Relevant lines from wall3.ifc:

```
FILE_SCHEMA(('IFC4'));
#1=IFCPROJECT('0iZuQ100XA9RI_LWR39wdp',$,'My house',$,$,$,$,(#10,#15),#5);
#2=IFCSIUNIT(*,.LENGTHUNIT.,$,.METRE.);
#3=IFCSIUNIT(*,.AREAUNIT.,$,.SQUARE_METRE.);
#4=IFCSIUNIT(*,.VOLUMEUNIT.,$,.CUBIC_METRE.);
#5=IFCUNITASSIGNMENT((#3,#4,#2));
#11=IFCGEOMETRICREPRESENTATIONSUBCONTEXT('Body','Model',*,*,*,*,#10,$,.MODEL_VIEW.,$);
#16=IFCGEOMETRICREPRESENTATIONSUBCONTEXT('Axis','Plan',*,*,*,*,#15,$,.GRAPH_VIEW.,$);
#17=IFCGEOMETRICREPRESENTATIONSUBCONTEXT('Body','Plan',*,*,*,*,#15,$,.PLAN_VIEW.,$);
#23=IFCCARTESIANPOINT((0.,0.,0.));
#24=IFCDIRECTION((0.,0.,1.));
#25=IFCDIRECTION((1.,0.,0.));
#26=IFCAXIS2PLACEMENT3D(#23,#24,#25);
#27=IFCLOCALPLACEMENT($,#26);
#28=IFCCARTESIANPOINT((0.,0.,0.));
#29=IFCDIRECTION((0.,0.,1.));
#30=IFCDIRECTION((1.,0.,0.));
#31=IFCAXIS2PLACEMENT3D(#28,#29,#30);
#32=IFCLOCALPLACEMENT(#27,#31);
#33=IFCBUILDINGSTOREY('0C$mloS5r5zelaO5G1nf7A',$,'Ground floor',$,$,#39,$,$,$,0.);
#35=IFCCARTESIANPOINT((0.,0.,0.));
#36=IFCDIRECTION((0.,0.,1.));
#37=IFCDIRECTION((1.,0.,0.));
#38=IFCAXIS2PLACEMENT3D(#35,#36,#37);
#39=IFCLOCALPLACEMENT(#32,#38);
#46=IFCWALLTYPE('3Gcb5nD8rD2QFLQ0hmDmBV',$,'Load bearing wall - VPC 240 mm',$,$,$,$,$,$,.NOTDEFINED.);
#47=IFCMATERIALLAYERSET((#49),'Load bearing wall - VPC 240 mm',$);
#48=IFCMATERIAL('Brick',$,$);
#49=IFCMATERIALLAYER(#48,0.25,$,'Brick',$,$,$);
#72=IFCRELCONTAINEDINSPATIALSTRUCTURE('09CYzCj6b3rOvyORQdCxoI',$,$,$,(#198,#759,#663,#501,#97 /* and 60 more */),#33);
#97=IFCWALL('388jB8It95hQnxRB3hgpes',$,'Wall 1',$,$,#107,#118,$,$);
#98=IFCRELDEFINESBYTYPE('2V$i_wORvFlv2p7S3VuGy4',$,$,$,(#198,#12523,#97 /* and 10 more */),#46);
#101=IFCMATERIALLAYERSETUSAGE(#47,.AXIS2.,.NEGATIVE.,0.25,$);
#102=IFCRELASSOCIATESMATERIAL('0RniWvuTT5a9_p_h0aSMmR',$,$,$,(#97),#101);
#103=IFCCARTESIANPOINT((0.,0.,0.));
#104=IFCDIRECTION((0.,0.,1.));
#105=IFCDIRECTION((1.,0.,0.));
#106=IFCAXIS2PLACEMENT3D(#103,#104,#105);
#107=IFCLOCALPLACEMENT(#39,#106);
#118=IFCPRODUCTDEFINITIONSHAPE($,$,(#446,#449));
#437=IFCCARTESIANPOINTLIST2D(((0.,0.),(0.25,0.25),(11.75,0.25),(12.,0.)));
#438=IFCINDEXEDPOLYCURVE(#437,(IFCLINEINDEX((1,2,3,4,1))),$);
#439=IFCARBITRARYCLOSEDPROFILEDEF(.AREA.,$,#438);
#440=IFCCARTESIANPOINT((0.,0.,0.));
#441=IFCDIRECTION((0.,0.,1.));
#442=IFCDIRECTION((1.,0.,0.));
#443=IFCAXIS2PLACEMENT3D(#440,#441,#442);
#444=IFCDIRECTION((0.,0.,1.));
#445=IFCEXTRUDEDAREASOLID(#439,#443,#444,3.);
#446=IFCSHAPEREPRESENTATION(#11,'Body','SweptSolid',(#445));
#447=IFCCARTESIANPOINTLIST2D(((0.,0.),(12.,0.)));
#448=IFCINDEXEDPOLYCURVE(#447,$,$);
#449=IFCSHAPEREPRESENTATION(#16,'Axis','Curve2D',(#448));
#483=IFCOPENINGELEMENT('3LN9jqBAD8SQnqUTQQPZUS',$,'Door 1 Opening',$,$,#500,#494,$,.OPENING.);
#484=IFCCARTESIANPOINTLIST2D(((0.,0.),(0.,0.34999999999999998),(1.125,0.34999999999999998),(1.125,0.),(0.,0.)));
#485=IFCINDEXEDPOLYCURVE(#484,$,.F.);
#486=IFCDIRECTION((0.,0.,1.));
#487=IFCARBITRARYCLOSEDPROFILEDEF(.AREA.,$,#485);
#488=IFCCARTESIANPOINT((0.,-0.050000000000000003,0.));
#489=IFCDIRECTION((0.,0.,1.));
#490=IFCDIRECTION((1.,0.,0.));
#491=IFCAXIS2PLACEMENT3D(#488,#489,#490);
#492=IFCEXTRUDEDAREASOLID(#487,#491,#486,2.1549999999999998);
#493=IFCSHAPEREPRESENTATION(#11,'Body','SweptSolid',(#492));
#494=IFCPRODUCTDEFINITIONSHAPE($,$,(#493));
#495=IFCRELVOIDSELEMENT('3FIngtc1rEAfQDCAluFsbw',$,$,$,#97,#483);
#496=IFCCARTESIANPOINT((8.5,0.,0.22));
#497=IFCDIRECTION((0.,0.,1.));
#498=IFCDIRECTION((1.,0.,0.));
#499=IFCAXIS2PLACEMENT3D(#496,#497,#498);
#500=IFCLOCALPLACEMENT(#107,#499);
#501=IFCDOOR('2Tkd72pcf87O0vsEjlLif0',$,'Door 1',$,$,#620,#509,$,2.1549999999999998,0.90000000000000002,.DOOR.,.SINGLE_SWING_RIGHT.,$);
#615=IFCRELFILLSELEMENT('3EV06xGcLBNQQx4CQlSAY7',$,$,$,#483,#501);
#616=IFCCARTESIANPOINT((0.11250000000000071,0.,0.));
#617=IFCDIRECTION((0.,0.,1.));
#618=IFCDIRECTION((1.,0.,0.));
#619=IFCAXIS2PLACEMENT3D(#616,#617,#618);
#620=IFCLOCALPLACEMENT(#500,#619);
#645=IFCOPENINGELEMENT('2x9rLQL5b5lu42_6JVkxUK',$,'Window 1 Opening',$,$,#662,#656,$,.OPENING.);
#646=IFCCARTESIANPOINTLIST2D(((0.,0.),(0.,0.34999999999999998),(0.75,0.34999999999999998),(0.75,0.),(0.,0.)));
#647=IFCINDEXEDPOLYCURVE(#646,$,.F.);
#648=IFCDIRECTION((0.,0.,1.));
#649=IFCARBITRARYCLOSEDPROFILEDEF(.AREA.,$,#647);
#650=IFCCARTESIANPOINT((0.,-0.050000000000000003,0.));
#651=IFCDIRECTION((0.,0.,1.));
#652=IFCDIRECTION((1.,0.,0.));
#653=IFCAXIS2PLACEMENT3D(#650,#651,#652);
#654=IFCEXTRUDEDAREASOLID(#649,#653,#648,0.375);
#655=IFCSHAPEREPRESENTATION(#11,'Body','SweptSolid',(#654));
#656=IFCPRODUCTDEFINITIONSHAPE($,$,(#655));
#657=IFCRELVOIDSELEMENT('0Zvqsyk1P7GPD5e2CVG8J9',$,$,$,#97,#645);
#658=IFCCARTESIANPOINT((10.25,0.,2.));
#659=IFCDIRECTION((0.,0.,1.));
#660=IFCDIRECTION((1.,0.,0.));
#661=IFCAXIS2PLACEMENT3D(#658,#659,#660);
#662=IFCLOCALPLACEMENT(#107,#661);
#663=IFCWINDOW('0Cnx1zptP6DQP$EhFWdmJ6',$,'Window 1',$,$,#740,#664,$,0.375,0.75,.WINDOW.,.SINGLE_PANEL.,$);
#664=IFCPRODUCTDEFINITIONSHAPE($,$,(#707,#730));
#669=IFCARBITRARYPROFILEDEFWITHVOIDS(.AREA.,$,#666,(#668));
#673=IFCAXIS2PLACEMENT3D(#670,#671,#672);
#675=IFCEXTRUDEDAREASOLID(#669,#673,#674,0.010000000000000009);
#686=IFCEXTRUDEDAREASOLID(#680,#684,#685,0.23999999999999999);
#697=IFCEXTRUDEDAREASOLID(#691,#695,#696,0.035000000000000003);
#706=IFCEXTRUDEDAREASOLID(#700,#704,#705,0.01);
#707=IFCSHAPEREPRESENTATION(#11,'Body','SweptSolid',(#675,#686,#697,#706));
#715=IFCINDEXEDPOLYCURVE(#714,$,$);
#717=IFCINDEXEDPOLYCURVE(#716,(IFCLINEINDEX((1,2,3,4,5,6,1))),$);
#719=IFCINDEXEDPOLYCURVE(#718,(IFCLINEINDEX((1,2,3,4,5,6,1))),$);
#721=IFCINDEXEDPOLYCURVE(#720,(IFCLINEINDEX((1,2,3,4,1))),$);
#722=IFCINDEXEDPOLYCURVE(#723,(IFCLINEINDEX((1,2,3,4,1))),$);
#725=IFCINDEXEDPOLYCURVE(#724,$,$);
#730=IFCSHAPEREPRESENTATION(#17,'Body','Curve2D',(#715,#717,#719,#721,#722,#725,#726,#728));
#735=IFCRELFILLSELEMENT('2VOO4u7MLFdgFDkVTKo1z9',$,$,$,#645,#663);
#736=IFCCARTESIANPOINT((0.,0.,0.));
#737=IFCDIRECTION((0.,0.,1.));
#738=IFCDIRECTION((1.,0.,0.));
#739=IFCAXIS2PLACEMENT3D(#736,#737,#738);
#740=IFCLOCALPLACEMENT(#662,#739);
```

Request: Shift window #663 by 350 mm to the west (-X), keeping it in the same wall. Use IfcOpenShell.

```python
import ifcopenshell
import ifcopenshell.api.geometry
import ifcopenshell.util.placement
import ifcopenshell.util.unit

model = ifcopenshell.open("wall3.ifc")
unit_scale = ifcopenshell.util.unit.calculate_unit_scale(model)

window = model.by_id(663)
opening = window.FillsVoids[0].RelatingOpeningElement
wall = opening.VoidsElements[0].RelatingBuildingElement

wall_matrix = ifcopenshell.util.placement.get_local_placement(wall.ObjectPlacement)
shift = wall_matrix[:3, 0] * -0.35 / unit_scale
before = ifcopenshell.util.placement.get_local_placement(window.ObjectPlacement)[:3, 3].copy()

# The window is placed relative to its opening, so it follows when the opening moves.
matrix = ifcopenshell.util.placement.get_local_placement(opening.ObjectPlacement)
matrix[:3, 3] += shift
ifcopenshell.api.geometry.edit_object_placement(
    model, product=opening, matrix=matrix, is_si=False, should_transform_children=True
)

after = ifcopenshell.util.placement.get_local_placement(window.ObjectPlacement)[:3, 3]
print("window moved by", (after - before).round(3) + 0.0)

model.write("wall3_updated.ifc")
```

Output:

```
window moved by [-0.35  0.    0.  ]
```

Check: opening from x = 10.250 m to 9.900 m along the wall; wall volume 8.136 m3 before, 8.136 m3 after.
